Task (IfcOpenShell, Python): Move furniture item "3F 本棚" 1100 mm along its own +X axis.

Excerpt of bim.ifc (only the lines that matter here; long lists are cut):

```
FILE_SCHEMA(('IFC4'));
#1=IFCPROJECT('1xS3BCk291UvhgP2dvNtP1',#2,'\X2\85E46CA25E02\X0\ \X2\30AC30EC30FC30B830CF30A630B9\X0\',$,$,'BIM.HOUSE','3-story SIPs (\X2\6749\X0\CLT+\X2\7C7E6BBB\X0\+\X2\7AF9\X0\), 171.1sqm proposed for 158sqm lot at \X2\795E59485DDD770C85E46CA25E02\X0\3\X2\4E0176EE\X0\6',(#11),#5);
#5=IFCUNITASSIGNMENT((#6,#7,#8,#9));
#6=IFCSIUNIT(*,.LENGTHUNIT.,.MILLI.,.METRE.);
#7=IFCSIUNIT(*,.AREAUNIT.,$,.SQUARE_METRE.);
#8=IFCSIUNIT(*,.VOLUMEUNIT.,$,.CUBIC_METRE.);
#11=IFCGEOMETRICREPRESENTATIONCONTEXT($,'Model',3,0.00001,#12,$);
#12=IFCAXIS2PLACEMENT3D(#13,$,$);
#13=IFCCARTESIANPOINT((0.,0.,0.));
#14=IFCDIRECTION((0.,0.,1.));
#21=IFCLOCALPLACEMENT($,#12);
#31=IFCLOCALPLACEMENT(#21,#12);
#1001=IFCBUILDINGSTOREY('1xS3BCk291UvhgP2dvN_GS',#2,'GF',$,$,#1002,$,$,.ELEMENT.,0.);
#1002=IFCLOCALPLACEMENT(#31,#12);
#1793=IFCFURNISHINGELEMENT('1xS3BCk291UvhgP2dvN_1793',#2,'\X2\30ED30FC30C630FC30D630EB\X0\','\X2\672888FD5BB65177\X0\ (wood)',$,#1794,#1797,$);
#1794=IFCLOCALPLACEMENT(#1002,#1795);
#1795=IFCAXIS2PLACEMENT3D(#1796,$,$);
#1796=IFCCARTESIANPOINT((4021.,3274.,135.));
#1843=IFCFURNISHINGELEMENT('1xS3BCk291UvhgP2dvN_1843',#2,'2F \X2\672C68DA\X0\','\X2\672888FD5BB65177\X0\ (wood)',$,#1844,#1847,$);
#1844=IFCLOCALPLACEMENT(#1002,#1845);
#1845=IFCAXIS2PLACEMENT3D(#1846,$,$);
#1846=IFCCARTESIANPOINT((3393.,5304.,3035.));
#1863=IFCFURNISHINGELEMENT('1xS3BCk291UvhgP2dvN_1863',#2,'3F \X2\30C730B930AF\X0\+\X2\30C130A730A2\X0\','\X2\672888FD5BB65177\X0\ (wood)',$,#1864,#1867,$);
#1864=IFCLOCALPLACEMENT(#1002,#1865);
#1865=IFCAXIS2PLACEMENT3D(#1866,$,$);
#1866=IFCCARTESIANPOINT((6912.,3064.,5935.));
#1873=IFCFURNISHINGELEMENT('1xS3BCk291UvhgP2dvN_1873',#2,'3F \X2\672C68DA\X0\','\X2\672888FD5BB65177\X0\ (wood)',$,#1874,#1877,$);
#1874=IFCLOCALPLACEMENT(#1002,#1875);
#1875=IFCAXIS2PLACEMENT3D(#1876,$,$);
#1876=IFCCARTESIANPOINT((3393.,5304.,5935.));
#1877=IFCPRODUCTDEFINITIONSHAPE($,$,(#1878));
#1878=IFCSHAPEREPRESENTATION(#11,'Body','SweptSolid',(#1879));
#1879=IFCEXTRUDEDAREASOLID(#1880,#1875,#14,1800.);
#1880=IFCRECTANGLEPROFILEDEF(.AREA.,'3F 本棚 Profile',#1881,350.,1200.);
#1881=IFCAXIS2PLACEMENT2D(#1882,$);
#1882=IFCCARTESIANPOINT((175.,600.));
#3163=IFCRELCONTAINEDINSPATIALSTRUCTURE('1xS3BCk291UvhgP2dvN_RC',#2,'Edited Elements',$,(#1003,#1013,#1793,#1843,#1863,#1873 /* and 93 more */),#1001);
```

```python
import ifcopenshell
import ifcopenshell.api.geometry
import ifcopenshell.util.placement
import ifcopenshell.util.unit

model = ifcopenshell.open("bim.ifc")
unit_scale = ifcopenshell.util.unit.calculate_unit_scale(model)

item = model.by_guid("1xS3BCk291UvhgP2dvN_1873")
matrix = ifcopenshell.util.placement.get_local_placement(item.ObjectPlacement)
matrix[:3, 3] += matrix[:3, 0] * 1.1 / unit_scale
ifcopenshell.api.geometry.edit_object_placement(model, product=item, matrix=matrix, is_si=False)

print(ifcopenshell.util.placement.get_local_placement(item.ObjectPlacement).round(3) + 0.0)

model.write("bim_edited.ifc")
```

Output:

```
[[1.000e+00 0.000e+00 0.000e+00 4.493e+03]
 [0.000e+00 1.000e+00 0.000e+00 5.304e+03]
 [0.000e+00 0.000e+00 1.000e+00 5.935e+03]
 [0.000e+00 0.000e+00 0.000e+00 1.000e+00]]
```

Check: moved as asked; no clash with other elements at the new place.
